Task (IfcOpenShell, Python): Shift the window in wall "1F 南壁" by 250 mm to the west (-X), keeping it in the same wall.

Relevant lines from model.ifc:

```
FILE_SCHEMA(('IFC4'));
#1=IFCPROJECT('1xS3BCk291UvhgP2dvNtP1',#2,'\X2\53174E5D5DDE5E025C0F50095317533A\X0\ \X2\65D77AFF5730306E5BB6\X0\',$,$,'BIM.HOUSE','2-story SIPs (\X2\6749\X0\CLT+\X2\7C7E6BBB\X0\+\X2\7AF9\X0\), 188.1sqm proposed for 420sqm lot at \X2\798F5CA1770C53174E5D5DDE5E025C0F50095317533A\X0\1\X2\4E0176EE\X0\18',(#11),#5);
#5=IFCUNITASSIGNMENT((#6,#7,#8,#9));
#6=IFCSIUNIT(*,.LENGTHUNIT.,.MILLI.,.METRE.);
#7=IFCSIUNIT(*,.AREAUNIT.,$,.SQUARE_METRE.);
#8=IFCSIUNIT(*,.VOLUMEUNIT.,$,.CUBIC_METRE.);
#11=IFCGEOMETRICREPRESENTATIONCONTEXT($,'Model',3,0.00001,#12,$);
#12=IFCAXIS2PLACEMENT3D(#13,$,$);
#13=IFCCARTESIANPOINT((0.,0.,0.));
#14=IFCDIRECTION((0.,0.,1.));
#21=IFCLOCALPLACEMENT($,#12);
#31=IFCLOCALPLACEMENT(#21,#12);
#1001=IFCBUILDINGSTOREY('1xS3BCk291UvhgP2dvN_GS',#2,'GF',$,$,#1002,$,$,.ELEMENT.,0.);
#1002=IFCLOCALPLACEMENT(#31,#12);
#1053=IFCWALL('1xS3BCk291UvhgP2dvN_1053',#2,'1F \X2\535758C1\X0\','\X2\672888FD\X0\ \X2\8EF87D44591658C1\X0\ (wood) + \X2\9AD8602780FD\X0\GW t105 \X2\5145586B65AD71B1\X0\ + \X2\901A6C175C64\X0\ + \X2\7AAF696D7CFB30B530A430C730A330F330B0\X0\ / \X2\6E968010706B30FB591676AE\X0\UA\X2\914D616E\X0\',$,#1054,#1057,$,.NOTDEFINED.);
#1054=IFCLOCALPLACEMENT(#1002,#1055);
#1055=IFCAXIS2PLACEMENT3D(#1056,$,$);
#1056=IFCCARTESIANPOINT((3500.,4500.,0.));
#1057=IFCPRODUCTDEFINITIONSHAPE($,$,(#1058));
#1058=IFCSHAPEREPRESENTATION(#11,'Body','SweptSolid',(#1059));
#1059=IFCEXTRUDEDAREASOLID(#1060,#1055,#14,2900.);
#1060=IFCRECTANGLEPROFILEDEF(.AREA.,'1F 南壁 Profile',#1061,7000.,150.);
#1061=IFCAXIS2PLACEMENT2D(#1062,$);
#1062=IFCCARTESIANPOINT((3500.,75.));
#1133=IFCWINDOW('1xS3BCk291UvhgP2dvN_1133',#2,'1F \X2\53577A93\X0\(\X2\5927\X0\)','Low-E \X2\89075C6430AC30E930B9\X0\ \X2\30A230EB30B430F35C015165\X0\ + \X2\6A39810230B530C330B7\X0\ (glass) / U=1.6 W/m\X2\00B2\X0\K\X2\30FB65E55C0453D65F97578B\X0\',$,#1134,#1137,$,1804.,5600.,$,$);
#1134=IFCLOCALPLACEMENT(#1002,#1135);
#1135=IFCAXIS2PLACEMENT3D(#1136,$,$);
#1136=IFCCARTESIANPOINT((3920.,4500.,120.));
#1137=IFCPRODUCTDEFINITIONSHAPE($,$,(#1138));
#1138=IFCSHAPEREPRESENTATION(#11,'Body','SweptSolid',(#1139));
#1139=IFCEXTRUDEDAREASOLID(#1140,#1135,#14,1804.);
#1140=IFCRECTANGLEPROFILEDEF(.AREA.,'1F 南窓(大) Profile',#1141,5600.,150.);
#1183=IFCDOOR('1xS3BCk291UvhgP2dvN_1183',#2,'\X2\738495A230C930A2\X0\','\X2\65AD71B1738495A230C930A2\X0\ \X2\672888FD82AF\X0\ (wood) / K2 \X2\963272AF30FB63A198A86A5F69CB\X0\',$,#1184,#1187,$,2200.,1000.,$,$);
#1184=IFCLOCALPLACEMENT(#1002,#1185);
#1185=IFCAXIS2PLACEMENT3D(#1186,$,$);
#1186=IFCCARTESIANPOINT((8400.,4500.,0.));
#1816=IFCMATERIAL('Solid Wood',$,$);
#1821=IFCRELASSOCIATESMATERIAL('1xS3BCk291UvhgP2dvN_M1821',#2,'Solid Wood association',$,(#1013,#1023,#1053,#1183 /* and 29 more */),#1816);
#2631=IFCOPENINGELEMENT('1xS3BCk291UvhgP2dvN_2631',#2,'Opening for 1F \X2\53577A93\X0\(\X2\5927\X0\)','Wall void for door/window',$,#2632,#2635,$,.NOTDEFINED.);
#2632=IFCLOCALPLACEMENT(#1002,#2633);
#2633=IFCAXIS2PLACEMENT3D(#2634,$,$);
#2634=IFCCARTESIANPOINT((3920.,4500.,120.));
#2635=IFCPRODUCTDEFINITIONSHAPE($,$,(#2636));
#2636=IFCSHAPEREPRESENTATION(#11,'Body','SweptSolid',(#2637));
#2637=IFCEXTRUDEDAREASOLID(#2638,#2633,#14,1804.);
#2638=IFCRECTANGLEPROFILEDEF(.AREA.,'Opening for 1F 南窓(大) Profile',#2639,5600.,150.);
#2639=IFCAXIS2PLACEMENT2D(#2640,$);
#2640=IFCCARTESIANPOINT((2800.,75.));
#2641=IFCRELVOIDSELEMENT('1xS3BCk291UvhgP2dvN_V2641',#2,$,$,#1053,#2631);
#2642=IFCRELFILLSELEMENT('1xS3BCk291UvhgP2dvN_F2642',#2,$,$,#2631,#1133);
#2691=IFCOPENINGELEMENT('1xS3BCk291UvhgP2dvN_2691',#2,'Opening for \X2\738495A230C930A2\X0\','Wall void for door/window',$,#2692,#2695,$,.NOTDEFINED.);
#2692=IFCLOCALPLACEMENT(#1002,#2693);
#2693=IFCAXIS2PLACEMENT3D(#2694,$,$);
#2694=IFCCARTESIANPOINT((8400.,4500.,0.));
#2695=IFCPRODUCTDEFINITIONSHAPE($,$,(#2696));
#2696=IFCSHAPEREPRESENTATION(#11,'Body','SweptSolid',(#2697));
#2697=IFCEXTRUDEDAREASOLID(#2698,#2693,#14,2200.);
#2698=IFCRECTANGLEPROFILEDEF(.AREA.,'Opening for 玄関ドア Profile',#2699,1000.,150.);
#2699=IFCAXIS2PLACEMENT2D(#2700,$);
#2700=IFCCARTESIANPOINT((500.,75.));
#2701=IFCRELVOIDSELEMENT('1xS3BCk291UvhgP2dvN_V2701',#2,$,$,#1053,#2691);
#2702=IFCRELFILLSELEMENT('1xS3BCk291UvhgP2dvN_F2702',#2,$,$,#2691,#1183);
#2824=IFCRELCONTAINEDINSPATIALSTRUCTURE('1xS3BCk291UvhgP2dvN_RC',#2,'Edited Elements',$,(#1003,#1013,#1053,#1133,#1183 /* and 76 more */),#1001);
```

```python
import ifcopenshell
import ifcopenshell.api.geometry
import ifcopenshell.util.placement

model = ifcopenshell.open("model.ifc")

window = model.by_guid("1xS3BCk291UvhgP2dvN_1133")
opening = window.FillsVoids[0].RelatingOpeningElement
wall = opening.VoidsElements[0].RelatingBuildingElement

wall_matrix = ifcopenshell.util.placement.get_local_placement(wall.ObjectPlacement)
shift = wall_matrix[:3, 0] * -250.0
before = ifcopenshell.util.placement.get_local_placement(window.ObjectPlacement)[:3, 3].copy()

# The window is not placed relative to its opening, so move both.
for product in (opening, window):
    matrix = ifcopenshell.util.placement.get_local_placement(product.ObjectPlacement)
    matrix[:3, 3] += shift
    ifcopenshell.api.geometry.edit_object_placement(model, product=product, matrix=matrix, is_si=False)

after = ifcopenshell.util.placement.get_local_placement(window.ObjectPlacement)[:3, 3]
print("window moved by", (after - before).round(3) + 0.0)

model.write("model_edited.ifc")
```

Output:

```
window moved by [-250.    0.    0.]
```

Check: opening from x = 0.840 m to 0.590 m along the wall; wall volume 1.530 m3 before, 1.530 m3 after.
